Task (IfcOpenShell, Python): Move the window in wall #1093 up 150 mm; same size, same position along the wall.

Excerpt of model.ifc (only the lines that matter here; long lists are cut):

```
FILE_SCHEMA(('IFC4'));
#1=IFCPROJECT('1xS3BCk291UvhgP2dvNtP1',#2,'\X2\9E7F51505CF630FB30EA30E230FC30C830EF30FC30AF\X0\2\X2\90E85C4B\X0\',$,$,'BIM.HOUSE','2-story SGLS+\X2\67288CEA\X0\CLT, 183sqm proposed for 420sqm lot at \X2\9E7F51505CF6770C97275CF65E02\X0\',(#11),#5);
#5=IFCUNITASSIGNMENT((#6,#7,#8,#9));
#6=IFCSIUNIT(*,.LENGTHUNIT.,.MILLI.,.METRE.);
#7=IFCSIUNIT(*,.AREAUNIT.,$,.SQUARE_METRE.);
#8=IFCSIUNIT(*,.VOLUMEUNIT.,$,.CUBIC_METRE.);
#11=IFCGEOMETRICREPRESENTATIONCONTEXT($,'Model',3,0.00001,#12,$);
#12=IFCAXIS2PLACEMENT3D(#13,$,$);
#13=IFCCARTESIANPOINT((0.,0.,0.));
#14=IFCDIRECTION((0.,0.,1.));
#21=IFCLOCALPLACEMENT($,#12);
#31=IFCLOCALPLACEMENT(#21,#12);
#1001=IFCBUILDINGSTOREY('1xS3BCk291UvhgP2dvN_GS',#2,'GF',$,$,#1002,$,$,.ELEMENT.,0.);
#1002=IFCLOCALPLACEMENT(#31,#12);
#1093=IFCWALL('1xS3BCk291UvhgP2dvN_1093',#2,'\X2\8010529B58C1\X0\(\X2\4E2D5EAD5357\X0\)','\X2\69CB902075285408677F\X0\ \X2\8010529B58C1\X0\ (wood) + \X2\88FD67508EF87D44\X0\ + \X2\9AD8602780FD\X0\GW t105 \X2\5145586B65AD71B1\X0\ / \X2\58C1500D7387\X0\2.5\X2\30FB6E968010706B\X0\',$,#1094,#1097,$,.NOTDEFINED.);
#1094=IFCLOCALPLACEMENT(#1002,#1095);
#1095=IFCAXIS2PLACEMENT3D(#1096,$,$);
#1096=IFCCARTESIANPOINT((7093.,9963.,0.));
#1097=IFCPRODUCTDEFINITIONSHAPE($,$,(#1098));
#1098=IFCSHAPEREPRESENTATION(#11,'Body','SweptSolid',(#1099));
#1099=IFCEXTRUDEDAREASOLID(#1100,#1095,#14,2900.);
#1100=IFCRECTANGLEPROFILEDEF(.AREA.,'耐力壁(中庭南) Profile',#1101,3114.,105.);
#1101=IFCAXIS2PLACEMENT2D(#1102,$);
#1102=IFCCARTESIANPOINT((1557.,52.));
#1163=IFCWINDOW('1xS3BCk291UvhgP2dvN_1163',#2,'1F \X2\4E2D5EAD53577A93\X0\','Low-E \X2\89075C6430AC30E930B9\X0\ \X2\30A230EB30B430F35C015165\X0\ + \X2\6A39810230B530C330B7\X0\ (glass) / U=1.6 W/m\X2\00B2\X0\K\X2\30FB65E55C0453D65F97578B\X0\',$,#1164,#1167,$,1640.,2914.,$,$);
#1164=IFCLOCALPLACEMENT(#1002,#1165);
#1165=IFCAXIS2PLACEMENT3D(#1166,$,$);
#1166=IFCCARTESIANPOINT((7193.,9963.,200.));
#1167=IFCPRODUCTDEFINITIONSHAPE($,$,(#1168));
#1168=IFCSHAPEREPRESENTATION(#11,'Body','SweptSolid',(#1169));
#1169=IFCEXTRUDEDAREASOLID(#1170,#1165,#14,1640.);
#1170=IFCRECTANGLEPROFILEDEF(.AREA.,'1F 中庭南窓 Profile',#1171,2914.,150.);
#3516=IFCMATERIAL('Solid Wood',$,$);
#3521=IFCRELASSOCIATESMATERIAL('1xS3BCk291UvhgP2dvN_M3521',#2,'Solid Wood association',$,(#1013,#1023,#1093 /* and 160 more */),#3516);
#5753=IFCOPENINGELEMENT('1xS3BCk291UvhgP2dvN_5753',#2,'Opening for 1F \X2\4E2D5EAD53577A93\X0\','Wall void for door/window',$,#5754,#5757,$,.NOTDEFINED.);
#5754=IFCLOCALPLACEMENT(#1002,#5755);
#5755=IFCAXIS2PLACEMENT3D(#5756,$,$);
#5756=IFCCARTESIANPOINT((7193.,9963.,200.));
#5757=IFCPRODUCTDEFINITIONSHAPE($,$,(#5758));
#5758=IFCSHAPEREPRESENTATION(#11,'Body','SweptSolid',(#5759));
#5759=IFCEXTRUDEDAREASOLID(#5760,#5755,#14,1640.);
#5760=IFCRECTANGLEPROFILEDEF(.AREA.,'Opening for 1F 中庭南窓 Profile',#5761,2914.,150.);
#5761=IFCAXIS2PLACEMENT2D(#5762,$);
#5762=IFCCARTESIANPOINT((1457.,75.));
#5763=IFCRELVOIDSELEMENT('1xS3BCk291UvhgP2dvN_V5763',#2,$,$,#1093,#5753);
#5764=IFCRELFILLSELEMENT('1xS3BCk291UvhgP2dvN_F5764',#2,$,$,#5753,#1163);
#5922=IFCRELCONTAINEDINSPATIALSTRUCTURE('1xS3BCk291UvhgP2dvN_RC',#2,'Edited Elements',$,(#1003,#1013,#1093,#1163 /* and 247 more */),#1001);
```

```python
import numpy as np
import ifcopenshell
import ifcopenshell.api.geometry
import ifcopenshell.util.placement
import ifcopenshell.util.unit

model = ifcopenshell.open("model.ifc")
unit_scale = ifcopenshell.util.unit.calculate_unit_scale(model)

window = model.by_guid("1xS3BCk291UvhgP2dvN_1163")
opening = window.FillsVoids[0].RelatingOpeningElement
dz = 0.15 / unit_scale

shift = np.array([0.0, 0.0, dz])
# The window is not placed relative to its opening, so move both.
for product in (opening, window):
    matrix = ifcopenshell.util.placement.get_local_placement(product.ObjectPlacement)
    matrix[:3, 3] += shift
    ifcopenshell.api.geometry.edit_object_placement(model, product=product, matrix=matrix, is_si=False)

print(f"moved by {dz * unit_scale:+.3f} m")

model.write("model_updated.ifc")
```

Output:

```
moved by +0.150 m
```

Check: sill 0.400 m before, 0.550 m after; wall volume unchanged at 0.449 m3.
